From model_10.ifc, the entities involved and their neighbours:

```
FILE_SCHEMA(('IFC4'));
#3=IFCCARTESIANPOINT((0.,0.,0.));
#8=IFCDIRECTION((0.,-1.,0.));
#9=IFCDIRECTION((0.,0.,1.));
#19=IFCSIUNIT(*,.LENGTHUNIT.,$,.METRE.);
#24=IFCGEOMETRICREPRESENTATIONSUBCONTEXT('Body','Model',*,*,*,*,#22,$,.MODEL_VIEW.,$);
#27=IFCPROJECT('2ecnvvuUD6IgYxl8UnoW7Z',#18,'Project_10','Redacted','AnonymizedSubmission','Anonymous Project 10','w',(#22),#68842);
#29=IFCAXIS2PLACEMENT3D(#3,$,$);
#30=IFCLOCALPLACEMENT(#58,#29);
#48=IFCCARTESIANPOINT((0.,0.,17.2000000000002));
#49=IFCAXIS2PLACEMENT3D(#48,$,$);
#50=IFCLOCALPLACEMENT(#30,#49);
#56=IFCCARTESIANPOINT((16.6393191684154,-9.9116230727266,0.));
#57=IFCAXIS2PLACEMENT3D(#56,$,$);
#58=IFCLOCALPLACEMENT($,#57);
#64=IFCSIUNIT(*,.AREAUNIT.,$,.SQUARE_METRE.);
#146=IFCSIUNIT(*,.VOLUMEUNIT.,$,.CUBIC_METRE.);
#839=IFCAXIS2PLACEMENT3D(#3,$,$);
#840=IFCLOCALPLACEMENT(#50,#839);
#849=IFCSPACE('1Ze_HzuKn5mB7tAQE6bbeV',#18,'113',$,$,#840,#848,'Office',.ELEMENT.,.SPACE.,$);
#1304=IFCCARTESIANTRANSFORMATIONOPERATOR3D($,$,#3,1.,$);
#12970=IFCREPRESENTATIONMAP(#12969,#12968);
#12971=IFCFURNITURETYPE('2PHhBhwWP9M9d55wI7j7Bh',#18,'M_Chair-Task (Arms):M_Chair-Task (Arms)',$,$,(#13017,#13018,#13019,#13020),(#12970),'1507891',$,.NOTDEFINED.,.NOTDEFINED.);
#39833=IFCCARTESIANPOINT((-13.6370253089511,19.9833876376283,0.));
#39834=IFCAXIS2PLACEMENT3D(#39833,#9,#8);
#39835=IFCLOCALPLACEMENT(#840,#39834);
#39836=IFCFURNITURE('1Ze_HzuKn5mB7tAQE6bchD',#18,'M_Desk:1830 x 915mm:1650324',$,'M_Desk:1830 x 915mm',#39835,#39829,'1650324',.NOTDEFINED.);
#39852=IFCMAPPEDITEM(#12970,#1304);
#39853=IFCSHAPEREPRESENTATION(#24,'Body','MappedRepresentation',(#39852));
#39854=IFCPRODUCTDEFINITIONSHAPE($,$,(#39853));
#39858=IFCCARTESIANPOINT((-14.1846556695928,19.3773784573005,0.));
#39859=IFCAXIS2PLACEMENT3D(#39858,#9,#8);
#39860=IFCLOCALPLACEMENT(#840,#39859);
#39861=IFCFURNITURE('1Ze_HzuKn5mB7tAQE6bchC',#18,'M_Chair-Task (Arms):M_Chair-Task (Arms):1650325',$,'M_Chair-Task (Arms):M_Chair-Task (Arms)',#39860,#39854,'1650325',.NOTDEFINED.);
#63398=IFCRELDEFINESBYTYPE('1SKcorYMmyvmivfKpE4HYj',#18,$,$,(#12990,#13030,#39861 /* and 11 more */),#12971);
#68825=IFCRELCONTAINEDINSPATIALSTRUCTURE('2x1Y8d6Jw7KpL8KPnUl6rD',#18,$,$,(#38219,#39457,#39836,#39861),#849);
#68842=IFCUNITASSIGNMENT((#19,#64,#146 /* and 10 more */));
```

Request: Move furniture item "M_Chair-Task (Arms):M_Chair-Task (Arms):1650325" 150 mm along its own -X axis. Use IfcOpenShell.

```python
import ifcopenshell
import ifcopenshell.api.geometry
import ifcopenshell.util.placement

model = ifcopenshell.open("model_10.ifc")

item = model.by_guid("1Ze_HzuKn5mB7tAQE6bchC")
matrix = ifcopenshell.util.placement.get_local_placement(item.ObjectPlacement)
matrix[:3, 3] -= matrix[:3, 0] * 0.15
ifcopenshell.api.geometry.edit_object_placement(model, product=item, matrix=matrix, is_si=False)

print(ifcopenshell.util.placement.get_local_placement(item.ObjectPlacement).round(3) + 0.0)

model.write("model_10_updated.ifc")
```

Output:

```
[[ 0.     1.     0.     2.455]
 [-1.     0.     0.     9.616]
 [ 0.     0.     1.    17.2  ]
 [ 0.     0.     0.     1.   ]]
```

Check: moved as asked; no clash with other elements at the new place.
